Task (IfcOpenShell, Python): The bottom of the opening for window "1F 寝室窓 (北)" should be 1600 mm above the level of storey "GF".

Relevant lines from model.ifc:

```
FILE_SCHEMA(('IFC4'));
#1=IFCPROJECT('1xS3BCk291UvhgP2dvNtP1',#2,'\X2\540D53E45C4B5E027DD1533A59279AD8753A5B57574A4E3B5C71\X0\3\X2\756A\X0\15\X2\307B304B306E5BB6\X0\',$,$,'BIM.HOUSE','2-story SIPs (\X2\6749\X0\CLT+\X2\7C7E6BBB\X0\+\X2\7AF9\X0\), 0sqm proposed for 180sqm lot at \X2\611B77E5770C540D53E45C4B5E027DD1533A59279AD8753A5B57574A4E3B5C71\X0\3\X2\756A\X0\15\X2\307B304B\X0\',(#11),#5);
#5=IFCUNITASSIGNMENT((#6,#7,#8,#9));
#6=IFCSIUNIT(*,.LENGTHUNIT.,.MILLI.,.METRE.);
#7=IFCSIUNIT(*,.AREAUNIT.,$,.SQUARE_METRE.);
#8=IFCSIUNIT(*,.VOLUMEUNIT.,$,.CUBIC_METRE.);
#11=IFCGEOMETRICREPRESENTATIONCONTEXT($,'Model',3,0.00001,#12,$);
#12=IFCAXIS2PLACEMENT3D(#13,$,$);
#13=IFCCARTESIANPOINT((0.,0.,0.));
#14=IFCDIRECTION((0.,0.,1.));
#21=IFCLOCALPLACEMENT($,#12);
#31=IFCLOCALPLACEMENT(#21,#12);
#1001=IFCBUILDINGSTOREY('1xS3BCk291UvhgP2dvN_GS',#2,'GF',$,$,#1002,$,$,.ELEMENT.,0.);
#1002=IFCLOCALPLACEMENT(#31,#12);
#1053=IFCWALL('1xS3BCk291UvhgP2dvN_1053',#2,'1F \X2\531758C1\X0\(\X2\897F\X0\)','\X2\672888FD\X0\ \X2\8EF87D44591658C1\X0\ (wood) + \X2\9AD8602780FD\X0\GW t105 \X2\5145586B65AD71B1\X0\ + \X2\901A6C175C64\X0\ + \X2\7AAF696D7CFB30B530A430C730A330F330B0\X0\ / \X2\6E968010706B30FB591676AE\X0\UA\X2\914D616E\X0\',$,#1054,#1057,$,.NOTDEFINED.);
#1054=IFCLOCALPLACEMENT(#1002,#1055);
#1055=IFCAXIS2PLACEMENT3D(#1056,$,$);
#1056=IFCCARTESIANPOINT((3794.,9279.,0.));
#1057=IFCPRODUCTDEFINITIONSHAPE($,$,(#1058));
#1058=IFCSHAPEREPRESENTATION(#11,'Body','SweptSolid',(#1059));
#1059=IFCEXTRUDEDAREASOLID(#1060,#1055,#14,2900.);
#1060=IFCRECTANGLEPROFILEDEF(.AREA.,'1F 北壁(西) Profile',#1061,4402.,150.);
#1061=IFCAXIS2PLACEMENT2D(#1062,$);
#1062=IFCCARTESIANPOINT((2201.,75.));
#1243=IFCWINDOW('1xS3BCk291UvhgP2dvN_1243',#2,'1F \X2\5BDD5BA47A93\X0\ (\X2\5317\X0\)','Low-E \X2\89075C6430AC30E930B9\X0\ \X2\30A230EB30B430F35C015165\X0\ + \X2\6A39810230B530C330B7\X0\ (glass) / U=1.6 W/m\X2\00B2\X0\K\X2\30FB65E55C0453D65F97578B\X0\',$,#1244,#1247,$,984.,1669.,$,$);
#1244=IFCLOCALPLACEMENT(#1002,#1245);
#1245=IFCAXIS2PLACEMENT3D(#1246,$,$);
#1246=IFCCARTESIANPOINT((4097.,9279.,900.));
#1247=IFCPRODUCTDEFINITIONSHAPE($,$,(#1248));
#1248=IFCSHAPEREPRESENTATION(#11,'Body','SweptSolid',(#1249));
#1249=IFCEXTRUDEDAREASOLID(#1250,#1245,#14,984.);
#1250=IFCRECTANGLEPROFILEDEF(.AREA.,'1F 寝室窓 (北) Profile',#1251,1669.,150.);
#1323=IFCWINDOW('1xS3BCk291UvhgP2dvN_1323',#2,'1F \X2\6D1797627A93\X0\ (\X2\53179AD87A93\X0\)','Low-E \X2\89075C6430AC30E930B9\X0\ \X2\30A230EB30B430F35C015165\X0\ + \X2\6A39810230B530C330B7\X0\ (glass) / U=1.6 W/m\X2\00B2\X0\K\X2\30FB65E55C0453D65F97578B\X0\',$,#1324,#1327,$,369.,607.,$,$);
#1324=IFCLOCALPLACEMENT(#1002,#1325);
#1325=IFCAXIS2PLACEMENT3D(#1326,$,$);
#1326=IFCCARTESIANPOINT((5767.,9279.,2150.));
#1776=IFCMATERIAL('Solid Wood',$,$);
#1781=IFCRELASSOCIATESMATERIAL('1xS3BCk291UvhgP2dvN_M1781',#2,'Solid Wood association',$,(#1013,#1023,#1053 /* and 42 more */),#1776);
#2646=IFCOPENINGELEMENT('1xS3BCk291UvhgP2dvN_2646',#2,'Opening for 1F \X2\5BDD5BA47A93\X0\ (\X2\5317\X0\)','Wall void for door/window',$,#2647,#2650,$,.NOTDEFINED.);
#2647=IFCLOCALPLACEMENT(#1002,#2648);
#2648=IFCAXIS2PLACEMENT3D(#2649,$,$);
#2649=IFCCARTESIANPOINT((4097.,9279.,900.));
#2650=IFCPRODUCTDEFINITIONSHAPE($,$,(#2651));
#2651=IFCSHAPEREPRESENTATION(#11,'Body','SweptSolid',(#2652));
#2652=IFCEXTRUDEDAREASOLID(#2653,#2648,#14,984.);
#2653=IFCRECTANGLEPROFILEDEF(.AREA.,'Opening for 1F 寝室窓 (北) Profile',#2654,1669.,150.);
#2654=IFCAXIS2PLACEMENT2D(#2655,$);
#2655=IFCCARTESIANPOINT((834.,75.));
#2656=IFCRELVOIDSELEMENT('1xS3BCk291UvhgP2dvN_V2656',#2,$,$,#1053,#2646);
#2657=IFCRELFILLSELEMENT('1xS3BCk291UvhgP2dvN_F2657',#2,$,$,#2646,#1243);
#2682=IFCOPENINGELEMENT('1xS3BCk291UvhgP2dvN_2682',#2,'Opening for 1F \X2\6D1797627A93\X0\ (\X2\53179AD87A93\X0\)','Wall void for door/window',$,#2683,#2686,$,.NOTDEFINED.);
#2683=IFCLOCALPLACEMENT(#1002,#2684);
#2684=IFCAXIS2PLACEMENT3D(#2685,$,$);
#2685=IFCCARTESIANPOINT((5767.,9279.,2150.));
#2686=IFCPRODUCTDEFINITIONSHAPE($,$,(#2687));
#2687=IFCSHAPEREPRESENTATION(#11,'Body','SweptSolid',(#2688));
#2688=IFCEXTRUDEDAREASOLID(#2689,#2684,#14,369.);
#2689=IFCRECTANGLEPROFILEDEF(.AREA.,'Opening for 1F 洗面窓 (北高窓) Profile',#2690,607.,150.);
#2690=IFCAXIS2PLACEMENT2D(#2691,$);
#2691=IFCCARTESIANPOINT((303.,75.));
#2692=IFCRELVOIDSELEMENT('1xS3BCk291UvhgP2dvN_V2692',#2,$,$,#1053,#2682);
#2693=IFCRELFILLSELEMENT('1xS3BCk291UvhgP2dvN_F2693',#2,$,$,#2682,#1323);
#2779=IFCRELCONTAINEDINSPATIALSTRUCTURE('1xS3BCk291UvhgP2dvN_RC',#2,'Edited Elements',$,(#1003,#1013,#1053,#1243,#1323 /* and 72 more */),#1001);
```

```python
import numpy as np
import ifcopenshell
import ifcopenshell.api.geometry
import ifcopenshell.geom
import ifcopenshell.util.element
import ifcopenshell.util.placement
import ifcopenshell.util.shape
import ifcopenshell.util.unit

model = ifcopenshell.open("model.ifc")
unit_scale = ifcopenshell.util.unit.calculate_unit_scale(model)

window = model.by_guid("1xS3BCk291UvhgP2dvN_1243")
opening = window.FillsVoids[0].RelatingOpeningElement
storey = ifcopenshell.util.element.get_container(window, ifc_class="IfcBuildingStorey")
level = ifcopenshell.util.placement.get_local_placement(storey.ObjectPlacement)[2, 3]

# The opening's origin need not be at the sill, so measure its lowest point.
shape = ifcopenshell.geom.create_shape(ifcopenshell.geom.settings(), opening)
bottom = ifcopenshell.util.shape.get_shape_bottom_elevation(shape, shape.geometry) / unit_scale
dz = level + 1.6 / unit_scale - bottom

shift = np.array([0.0, 0.0, dz])
# The window is not placed relative to its opening, so move both.
for product in (opening, window):
    matrix = ifcopenshell.util.placement.get_local_placement(product.ObjectPlacement)
    matrix[:3, 3] += shift
    ifcopenshell.api.geometry.edit_object_placement(model, product=product, matrix=matrix, is_si=False)

print(f"moved by {dz * unit_scale:+.3f} m")

model.write("model_v2.ifc")
```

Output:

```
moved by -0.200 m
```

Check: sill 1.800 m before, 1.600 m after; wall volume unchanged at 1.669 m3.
